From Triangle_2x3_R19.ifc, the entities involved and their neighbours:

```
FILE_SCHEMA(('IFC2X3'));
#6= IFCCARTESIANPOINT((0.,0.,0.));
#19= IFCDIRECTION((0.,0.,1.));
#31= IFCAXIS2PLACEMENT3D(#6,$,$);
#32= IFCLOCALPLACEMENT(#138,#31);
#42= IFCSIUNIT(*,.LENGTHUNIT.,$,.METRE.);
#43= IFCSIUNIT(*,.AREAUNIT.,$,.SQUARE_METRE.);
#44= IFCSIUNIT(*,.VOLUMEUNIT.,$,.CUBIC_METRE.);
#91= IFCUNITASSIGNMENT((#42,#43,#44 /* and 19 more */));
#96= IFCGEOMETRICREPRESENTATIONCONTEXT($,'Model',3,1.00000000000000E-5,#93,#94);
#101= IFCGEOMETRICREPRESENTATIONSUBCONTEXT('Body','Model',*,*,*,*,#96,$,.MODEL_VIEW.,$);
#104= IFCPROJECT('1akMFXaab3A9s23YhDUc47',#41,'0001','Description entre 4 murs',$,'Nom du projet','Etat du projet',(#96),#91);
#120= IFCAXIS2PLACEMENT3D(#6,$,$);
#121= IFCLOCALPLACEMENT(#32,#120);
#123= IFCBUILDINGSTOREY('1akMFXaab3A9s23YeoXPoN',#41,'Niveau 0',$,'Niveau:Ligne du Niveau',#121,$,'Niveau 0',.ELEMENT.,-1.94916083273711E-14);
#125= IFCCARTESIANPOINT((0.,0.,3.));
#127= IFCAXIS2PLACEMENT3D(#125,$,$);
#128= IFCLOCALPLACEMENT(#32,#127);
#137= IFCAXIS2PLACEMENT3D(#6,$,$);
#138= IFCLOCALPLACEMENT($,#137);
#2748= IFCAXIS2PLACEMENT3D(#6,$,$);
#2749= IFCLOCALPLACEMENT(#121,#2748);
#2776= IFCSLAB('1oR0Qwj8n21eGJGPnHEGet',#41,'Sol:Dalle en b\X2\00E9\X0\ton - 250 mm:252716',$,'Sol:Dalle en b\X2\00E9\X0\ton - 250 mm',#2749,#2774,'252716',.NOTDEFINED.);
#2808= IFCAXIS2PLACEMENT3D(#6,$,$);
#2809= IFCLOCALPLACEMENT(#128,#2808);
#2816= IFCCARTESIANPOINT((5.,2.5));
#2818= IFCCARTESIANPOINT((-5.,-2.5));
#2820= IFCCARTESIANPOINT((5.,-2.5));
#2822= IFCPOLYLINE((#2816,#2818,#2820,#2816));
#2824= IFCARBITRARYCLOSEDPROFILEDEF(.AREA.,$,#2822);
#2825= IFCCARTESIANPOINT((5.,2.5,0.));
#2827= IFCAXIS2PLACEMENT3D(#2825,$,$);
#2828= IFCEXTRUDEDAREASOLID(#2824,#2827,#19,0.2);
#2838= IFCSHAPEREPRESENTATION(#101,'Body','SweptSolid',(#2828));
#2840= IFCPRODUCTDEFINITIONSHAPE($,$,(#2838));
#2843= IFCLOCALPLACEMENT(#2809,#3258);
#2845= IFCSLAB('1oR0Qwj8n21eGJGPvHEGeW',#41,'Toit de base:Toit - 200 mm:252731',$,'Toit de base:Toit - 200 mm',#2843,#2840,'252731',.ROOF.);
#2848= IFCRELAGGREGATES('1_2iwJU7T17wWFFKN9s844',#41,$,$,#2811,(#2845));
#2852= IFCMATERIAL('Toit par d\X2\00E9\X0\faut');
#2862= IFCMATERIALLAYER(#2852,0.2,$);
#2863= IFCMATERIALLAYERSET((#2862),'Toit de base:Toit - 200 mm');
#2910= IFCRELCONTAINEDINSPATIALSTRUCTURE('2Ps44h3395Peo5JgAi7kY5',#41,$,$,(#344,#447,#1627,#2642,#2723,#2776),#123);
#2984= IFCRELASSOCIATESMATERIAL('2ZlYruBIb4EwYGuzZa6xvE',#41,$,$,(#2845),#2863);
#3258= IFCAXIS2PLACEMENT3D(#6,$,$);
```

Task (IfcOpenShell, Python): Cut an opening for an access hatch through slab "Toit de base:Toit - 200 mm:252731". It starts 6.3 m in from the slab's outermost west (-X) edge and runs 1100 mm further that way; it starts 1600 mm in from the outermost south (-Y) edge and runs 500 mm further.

```python
import numpy as np
import ifcopenshell
import ifcopenshell.api.feature
import ifcopenshell.api.geometry
import ifcopenshell.api.root
import ifcopenshell.geom
import ifcopenshell.util.placement
import ifcopenshell.util.representation
import ifcopenshell.util.shape
import ifcopenshell.util.unit

model = ifcopenshell.open("Triangle_2x3_R19.ifc")
unit_scale = ifcopenshell.util.unit.calculate_unit_scale(model)
settings = ifcopenshell.geom.settings()


def volume(element):
    """Net volume in cubic metres, openings subtracted."""
    shape = ifcopenshell.geom.create_shape(settings, element)
    return ifcopenshell.util.shape.get_volume(shape.geometry)


slab = model.by_id(2845)
before = volume(slab)

# Extent in the slab's own axes, in metres. The edges named are its -X and -Y sides.
slab_shape = ifcopenshell.geom.create_shape(settings, slab)
vertices = ifcopenshell.util.shape.get_vertices(slab_shape.geometry)
x_min, y_min, bottom = vertices.min(axis=0)
top = vertices[:, 2].max()

opening = ifcopenshell.api.root.create_entity(model, ifc_class="IfcOpeningElement", name="Access hatch opening")
context = ifcopenshell.util.representation.get_context(model, "Model", "Body", "MODEL_VIEW")
width, depth = 1.1, 0.5
outline = [(0.0, 0.0), (width, 0.0), (width, depth), (0.0, depth), (0.0, 0.0)]
# Overshoot both faces by 50 mm so the cut is clean.
shape = ifcopenshell.api.geometry.add_slab_representation(
    model, context=context, depth=top - bottom + 0.1, polyline=outline
)
ifcopenshell.api.geometry.assign_representation(model, product=opening, representation=shape)

matrix = ifcopenshell.util.placement.get_local_placement(slab.ObjectPlacement)
matrix[:, 3] = matrix @ np.append(np.array([x_min + 6.3, y_min + 1.6, bottom - 0.05]) / unit_scale, 1.0)
ifcopenshell.api.geometry.edit_object_placement(model, product=opening, matrix=matrix, is_si=False)
ifcopenshell.api.feature.add_feature(model, feature=opening, element=slab)

after = volume(slab)

print(f"slab volume {before:.3f} -> {after:.3f} m3")

model.write("Triangle_2x3_R19_edited.ifc")
```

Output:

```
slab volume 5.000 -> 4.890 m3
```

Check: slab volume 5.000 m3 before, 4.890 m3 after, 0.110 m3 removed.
